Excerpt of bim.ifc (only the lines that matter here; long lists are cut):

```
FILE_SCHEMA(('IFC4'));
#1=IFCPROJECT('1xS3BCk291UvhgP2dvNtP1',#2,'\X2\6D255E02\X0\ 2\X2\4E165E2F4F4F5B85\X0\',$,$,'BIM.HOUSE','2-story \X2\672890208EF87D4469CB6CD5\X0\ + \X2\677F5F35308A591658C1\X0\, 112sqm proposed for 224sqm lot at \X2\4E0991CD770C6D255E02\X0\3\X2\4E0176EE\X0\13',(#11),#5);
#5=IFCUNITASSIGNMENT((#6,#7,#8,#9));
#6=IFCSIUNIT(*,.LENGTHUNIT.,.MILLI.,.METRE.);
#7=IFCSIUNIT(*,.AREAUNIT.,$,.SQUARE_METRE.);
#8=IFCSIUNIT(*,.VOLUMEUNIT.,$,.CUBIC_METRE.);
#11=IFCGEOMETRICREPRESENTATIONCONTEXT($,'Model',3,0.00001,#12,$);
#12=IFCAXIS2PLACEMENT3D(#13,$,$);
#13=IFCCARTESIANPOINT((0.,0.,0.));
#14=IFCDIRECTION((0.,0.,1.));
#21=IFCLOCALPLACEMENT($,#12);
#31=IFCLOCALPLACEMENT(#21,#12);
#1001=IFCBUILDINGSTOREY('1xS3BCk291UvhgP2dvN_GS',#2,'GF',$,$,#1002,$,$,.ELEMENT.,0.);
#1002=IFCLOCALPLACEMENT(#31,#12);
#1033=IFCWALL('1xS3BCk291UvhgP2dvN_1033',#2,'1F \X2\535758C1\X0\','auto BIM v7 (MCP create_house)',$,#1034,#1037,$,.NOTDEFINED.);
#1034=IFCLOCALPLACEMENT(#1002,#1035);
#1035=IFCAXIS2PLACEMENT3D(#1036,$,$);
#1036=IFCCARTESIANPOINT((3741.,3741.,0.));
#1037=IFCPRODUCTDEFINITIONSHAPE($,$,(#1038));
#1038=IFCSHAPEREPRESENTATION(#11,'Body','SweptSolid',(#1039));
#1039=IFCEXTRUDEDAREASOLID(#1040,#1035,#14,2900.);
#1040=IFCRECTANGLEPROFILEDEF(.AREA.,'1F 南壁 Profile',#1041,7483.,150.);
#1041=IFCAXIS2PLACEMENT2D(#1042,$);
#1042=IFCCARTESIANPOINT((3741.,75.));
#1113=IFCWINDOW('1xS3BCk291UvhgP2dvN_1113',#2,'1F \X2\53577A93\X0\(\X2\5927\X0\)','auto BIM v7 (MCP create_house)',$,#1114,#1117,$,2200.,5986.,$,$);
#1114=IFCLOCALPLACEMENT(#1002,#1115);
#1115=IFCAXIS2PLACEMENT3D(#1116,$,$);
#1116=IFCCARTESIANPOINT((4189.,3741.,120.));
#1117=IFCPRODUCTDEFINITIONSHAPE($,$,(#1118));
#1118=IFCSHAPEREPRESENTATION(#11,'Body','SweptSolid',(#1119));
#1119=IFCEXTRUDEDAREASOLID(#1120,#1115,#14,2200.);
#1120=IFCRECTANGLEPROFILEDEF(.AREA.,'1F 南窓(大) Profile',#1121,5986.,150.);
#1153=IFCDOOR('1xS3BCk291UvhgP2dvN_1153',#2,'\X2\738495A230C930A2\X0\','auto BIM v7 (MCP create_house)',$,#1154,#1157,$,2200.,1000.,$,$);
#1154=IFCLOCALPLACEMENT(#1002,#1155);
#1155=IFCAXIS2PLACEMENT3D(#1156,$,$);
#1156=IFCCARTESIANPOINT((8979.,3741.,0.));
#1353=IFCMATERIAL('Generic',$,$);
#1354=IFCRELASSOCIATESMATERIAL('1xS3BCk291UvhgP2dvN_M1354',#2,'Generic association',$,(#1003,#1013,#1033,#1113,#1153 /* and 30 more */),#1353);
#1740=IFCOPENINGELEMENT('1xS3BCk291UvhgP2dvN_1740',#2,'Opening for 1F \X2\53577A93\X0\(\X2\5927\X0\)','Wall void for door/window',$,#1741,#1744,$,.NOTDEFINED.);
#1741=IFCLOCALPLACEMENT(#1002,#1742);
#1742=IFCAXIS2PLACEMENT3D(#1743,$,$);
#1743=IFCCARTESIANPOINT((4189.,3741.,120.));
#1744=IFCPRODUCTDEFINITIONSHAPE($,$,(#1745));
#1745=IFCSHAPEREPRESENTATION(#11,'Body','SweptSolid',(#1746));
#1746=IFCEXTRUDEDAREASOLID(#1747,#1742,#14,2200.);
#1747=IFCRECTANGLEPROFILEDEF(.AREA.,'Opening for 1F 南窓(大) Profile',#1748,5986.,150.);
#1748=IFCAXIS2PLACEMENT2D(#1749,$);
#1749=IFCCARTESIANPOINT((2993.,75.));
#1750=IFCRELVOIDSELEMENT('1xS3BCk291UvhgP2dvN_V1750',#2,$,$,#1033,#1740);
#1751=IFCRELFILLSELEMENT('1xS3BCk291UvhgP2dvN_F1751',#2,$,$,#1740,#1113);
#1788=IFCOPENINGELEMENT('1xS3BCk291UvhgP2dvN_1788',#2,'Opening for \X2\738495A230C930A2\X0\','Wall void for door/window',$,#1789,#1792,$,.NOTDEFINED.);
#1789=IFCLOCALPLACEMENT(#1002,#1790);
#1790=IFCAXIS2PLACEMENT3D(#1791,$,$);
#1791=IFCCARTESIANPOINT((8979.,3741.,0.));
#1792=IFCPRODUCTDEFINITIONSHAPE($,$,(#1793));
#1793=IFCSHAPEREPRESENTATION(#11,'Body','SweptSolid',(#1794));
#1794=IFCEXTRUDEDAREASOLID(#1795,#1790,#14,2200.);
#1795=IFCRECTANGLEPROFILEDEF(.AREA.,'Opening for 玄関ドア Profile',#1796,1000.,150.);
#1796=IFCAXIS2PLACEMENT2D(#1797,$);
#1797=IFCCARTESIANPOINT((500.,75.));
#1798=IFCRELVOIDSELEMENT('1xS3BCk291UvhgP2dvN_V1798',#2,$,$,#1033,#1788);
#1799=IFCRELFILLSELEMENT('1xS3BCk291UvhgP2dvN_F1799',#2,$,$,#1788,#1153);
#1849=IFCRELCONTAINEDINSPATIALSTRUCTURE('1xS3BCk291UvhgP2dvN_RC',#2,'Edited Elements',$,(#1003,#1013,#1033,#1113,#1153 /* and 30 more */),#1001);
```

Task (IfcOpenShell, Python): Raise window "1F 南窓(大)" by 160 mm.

```python
import numpy as np
import ifcopenshell
import ifcopenshell.api.geometry
import ifcopenshell.util.placement
import ifcopenshell.util.unit

model = ifcopenshell.open("bim.ifc")
unit_scale = ifcopenshell.util.unit.calculate_unit_scale(model)

window = model.by_id(1113)
opening = window.FillsVoids[0].RelatingOpeningElement
dz = 0.16 / unit_scale

shift = np.array([0.0, 0.0, dz])
# The window is not placed relative to its opening, so move both.
for product in (opening, window):
    matrix = ifcopenshell.util.placement.get_local_placement(product.ObjectPlacement)
    matrix[:3, 3] += shift
    ifcopenshell.api.geometry.edit_object_placement(model, product=product, matrix=matrix, is_si=False)

print(f"moved by {dz * unit_scale:+.3f} m")

model.write("bim_rev.ifc")
```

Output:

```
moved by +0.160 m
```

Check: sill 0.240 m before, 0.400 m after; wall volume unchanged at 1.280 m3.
